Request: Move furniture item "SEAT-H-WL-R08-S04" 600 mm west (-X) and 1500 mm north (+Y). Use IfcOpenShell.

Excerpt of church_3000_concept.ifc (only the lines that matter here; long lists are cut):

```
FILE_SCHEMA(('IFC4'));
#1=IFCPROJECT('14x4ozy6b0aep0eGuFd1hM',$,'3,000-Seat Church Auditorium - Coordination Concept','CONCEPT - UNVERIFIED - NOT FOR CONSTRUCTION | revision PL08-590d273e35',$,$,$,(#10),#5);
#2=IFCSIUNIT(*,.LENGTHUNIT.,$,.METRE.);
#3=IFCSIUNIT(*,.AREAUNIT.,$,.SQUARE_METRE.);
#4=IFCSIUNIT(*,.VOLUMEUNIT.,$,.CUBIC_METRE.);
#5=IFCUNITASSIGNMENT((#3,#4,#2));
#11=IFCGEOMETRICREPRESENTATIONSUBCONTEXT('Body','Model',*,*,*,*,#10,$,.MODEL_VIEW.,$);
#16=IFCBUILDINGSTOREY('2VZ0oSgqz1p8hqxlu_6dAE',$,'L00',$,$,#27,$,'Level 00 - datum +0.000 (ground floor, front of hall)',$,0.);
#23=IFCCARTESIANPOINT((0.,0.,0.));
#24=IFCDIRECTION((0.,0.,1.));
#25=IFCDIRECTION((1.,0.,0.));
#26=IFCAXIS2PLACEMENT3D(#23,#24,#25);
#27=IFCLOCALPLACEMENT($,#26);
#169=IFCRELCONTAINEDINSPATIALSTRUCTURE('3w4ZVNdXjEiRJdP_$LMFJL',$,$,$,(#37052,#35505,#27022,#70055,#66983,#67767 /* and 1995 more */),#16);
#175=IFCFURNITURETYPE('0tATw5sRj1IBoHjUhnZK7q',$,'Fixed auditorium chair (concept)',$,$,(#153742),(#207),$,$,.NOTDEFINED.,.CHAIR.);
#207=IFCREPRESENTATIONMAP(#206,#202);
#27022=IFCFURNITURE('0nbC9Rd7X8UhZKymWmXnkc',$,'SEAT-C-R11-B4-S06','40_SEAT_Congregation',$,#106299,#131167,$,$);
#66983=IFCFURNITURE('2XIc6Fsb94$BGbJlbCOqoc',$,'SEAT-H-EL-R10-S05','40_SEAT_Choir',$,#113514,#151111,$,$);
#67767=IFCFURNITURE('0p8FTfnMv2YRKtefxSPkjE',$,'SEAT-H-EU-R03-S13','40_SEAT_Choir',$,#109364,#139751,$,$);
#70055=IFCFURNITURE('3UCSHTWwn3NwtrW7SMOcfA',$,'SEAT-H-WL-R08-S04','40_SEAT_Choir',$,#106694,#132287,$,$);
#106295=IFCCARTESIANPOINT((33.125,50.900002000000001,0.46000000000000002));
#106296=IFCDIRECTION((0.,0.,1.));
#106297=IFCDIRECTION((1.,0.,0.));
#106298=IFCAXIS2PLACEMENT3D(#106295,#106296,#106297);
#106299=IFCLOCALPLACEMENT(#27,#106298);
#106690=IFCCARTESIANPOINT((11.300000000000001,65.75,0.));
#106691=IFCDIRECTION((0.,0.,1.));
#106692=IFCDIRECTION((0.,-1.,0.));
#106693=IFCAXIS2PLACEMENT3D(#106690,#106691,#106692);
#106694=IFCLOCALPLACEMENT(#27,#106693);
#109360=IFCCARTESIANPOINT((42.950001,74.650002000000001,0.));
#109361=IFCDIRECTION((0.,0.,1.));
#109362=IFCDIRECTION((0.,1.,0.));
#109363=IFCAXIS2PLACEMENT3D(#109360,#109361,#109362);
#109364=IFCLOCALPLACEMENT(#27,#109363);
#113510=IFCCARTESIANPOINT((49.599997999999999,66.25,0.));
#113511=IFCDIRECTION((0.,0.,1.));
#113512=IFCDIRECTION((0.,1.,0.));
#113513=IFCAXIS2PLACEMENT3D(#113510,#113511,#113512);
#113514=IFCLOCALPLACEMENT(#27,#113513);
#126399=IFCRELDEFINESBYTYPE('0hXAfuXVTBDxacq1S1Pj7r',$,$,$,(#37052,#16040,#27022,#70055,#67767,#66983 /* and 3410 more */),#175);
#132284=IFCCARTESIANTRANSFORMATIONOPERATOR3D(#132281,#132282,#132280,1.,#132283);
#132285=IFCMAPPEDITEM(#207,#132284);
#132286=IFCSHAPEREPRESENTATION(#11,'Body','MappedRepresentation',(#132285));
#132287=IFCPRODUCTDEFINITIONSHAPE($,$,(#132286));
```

```python
import ifcopenshell
import ifcopenshell.api.geometry
import ifcopenshell.util.placement
import ifcopenshell.util.unit

model = ifcopenshell.open("church_3000_concept.ifc")
unit_scale = ifcopenshell.util.unit.calculate_unit_scale(model)

item = model.by_guid("3UCSHTWwn3NwtrW7SMOcfA")
matrix = ifcopenshell.util.placement.get_local_placement(item.ObjectPlacement)
matrix[0, 3] -= 0.6 / unit_scale
matrix[1, 3] += 1.5 / unit_scale
ifcopenshell.api.geometry.edit_object_placement(model, product=item, matrix=matrix, is_si=False)

print(ifcopenshell.util.placement.get_local_placement(item.ObjectPlacement).round(3) + 0.0)

model.write("church_3000_concept_updated.ifc")
```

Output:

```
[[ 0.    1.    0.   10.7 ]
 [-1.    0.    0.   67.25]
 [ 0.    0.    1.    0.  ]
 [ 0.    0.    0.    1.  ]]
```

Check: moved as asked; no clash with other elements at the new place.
